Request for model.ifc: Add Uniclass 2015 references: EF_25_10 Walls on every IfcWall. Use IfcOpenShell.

First a look at what the model holds.

```python
import ifcopenshell

model = ifcopenshell.open("model.ifc")
print(model.schema)
print("classifications:", [c.Name for c in model.by_type("IfcClassification")])
for ifc_class in ("IfcDoor", "IfcRoof", "IfcStair", "IfcWall", "IfcWindow"):
    print(ifc_class, len(model.by_type(ifc_class)))
```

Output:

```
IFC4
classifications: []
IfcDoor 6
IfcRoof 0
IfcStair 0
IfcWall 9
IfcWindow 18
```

```python
import ifcopenshell
import ifcopenshell.api.classification

model = ifcopenshell.open("model.ifc")

system = ifcopenshell.api.classification.add_classification(model, classification="Uniclass 2015")

codes = {
    "IfcWall": ("EF_25_10", "Walls"),
}
for ifc_class, (code, name) in codes.items():
    products = model.by_type(ifc_class)
    ifcopenshell.api.classification.add_reference(
        model, products=products, classification=system, identification=code, name=name
    )
    print(code, len(products))

model.write("model-out.ifc")
```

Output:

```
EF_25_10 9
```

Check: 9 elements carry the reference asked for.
